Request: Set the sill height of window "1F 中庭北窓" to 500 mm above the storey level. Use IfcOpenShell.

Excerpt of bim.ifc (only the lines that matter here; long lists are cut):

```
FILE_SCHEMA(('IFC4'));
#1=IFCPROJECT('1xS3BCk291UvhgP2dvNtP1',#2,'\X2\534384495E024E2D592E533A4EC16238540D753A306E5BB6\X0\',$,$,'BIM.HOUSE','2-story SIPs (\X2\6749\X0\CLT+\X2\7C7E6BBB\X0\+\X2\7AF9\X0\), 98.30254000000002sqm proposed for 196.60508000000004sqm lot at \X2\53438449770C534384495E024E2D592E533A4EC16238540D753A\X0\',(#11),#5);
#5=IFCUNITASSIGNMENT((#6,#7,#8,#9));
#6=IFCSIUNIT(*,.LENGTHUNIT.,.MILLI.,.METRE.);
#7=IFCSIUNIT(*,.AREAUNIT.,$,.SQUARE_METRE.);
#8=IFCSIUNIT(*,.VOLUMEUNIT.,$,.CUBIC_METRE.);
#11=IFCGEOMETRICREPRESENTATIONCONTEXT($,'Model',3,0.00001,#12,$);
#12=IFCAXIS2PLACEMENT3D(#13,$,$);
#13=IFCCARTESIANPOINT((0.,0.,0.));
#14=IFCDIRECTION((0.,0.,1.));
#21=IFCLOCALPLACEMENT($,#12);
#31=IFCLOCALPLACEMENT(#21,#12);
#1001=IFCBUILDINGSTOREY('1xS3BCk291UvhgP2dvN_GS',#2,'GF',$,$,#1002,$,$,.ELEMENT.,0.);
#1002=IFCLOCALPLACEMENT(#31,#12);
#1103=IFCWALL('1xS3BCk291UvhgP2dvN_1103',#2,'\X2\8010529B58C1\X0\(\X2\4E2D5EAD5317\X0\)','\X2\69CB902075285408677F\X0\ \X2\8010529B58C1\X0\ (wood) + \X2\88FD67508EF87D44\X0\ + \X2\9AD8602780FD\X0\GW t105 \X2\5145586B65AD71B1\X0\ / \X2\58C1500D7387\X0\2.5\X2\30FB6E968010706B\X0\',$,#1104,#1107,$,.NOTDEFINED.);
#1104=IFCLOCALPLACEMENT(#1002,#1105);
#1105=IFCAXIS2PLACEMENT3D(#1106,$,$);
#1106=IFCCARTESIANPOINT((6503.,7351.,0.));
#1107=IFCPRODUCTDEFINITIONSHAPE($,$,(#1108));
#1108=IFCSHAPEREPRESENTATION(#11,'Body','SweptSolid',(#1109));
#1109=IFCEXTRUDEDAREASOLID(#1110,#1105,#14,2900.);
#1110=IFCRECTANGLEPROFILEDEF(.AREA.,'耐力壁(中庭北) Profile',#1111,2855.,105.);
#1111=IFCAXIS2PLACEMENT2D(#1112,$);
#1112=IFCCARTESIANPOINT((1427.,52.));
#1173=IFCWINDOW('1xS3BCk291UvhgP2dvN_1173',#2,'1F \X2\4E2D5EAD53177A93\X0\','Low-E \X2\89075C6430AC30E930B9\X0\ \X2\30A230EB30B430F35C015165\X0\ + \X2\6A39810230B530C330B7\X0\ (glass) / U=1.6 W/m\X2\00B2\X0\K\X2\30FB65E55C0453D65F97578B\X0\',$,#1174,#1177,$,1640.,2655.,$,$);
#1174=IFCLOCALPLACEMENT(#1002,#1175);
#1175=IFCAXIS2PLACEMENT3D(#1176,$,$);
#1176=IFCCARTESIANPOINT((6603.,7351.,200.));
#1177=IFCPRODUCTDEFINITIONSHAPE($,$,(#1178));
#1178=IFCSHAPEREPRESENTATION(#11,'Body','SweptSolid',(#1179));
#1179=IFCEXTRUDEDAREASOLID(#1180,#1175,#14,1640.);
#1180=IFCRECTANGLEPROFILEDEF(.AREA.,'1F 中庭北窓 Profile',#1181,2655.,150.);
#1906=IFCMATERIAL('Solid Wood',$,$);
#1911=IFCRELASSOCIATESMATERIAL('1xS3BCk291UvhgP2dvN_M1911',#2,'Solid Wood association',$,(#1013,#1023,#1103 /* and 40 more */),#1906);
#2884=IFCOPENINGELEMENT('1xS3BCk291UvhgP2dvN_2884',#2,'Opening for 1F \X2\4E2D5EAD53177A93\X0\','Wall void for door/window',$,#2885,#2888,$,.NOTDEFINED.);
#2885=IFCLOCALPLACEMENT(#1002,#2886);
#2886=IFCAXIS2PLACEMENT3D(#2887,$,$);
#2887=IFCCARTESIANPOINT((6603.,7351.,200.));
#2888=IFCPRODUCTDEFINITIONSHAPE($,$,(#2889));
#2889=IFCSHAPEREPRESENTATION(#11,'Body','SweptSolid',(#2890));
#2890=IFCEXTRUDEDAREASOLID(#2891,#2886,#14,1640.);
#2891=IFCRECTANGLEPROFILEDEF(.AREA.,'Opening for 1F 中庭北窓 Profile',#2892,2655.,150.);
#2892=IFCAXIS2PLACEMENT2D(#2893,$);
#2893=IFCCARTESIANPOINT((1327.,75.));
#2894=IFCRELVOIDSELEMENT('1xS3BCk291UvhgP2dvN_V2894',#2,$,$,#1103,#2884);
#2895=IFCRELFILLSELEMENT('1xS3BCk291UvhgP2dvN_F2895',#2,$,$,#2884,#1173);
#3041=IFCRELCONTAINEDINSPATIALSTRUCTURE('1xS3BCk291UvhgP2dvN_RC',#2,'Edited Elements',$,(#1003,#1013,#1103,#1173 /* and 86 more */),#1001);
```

```python
import numpy as np
import ifcopenshell
import ifcopenshell.api.geometry
import ifcopenshell.geom
import ifcopenshell.util.element
import ifcopenshell.util.placement
import ifcopenshell.util.shape
import ifcopenshell.util.unit

model = ifcopenshell.open("bim.ifc")
unit_scale = ifcopenshell.util.unit.calculate_unit_scale(model)

window = model.by_id(1173)
opening = window.FillsVoids[0].RelatingOpeningElement
storey = ifcopenshell.util.element.get_container(window, ifc_class="IfcBuildingStorey")
level = ifcopenshell.util.placement.get_local_placement(storey.ObjectPlacement)[2, 3]

# The opening's origin need not be at the sill, so measure its lowest point.
shape = ifcopenshell.geom.create_shape(ifcopenshell.geom.settings(), opening)
bottom = ifcopenshell.util.shape.get_shape_bottom_elevation(shape, shape.geometry) / unit_scale
dz = level + 0.5 / unit_scale - bottom

shift = np.array([0.0, 0.0, dz])
# The window is not placed relative to its opening, so move both.
for product in (opening, window):
    matrix = ifcopenshell.util.placement.get_local_placement(product.ObjectPlacement)
    matrix[:3, 3] += shift
    ifcopenshell.api.geometry.edit_object_placement(model, product=product, matrix=matrix, is_si=False)

print(f"moved by {dz * unit_scale:+.3f} m")

model.write("bim_v2.ifc")
```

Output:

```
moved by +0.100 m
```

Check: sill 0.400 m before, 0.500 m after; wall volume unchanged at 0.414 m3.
